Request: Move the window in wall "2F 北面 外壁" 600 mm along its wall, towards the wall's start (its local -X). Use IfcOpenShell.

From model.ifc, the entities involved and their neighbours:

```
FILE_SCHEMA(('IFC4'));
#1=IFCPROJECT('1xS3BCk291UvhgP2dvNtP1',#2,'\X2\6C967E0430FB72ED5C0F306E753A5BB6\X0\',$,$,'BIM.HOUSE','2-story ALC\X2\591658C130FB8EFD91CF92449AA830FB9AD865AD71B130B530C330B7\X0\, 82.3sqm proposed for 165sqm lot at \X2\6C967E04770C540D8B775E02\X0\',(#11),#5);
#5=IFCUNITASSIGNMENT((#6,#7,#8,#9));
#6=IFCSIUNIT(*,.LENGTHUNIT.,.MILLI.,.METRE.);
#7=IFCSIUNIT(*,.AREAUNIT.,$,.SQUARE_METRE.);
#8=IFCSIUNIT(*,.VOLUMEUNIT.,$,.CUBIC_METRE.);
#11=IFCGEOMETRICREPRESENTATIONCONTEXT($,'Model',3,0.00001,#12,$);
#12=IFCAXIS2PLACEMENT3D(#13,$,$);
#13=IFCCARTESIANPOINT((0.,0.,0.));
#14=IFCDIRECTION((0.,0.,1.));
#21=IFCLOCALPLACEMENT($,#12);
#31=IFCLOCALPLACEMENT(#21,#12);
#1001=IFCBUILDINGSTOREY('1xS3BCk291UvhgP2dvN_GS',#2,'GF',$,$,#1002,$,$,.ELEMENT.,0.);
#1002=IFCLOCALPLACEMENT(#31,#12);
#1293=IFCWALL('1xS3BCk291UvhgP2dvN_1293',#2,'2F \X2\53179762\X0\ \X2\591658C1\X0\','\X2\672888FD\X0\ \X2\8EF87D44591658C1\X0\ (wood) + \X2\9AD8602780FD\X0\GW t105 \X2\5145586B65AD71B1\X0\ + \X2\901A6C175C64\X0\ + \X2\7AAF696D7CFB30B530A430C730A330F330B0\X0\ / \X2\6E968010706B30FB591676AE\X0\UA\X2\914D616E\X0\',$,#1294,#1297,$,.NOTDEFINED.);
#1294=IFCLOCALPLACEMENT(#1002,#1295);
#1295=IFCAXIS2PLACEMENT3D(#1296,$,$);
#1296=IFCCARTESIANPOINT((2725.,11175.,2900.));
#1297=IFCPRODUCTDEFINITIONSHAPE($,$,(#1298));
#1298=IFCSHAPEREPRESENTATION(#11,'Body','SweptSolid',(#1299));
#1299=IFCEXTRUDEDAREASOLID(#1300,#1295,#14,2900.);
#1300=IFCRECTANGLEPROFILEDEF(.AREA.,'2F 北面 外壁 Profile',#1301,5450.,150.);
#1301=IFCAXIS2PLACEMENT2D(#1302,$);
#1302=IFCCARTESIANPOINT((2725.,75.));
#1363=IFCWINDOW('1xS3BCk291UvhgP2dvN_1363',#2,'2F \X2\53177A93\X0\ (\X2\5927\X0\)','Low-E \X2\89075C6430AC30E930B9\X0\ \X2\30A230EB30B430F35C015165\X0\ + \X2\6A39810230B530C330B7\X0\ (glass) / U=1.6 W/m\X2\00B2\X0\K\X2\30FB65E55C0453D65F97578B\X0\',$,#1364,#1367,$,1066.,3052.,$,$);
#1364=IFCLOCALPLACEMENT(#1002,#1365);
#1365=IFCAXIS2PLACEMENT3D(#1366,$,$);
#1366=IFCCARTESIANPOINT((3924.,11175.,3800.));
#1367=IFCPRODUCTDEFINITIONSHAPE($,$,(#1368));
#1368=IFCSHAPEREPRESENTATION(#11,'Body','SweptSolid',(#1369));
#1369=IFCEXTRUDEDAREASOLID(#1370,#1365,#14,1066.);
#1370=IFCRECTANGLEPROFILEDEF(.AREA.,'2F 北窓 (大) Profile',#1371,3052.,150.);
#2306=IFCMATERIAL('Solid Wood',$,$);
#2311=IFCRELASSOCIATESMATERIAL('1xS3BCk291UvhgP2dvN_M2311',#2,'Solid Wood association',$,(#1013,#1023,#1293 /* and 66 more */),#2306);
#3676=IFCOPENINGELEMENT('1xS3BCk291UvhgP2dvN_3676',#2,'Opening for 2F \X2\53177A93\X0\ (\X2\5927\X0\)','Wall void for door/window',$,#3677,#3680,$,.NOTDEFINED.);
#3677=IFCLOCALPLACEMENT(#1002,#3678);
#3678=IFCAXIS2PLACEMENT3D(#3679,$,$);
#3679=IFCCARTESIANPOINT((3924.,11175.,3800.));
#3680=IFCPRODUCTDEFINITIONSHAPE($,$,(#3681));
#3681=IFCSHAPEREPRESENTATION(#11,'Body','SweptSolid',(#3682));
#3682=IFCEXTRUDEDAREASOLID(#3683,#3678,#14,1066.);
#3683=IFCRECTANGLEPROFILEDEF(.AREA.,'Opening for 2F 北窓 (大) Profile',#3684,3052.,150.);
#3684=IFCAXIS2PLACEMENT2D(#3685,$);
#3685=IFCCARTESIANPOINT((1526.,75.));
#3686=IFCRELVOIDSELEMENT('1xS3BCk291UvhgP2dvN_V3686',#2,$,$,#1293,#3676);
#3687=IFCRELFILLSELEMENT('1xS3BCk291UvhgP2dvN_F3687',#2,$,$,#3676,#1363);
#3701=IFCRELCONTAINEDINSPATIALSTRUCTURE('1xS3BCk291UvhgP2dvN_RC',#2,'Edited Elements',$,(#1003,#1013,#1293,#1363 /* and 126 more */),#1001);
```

```python
import ifcopenshell
import ifcopenshell.api.geometry
import ifcopenshell.util.placement

model = ifcopenshell.open("model.ifc")

window = model.by_id(1363)
opening = window.FillsVoids[0].RelatingOpeningElement
wall = opening.VoidsElements[0].RelatingBuildingElement

wall_matrix = ifcopenshell.util.placement.get_local_placement(wall.ObjectPlacement)
shift = wall_matrix[:3, 0] * -600.0
before = ifcopenshell.util.placement.get_local_placement(window.ObjectPlacement)[:3, 3].copy()

# The window is not placed relative to its opening, so move both.
for product in (opening, window):
    matrix = ifcopenshell.util.placement.get_local_placement(product.ObjectPlacement)
    matrix[:3, 3] += shift
    ifcopenshell.api.geometry.edit_object_placement(model, product=product, matrix=matrix, is_si=False)

after = ifcopenshell.util.placement.get_local_placement(window.ObjectPlacement)[:3, 3]
print("window moved by", (after - before).round(3) + 0.0)

model.write("model_updated.ifc")
```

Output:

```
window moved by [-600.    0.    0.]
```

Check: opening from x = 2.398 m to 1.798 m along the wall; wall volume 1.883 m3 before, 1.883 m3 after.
